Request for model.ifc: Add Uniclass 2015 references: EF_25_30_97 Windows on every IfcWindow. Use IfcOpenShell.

First a look at what the model holds.

```python
import ifcopenshell

model = ifcopenshell.open("model.ifc")
print(model.schema)
print("classifications:", [c.Name for c in model.by_type("IfcClassification")])
for ifc_class in ("IfcDoor", "IfcRoof", "IfcStair", "IfcWall", "IfcWindow"):
    print(ifc_class, len(model.by_type(ifc_class)))
```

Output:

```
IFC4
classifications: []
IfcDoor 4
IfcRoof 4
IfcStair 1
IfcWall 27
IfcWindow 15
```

```python
import ifcopenshell
import ifcopenshell.api.classification

model = ifcopenshell.open("model.ifc")

system = ifcopenshell.api.classification.add_classification(model, classification="Uniclass 2015")

codes = {
    "IfcWindow": ("EF_25_30_97", "Windows"),
}
for ifc_class, (code, name) in codes.items():
    products = model.by_type(ifc_class)
    ifcopenshell.api.classification.add_reference(
        model, products=products, classification=system, identification=code, name=name
    )
    print(code, len(products))

model.write("model_updated.ifc")
```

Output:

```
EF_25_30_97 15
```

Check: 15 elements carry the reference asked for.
